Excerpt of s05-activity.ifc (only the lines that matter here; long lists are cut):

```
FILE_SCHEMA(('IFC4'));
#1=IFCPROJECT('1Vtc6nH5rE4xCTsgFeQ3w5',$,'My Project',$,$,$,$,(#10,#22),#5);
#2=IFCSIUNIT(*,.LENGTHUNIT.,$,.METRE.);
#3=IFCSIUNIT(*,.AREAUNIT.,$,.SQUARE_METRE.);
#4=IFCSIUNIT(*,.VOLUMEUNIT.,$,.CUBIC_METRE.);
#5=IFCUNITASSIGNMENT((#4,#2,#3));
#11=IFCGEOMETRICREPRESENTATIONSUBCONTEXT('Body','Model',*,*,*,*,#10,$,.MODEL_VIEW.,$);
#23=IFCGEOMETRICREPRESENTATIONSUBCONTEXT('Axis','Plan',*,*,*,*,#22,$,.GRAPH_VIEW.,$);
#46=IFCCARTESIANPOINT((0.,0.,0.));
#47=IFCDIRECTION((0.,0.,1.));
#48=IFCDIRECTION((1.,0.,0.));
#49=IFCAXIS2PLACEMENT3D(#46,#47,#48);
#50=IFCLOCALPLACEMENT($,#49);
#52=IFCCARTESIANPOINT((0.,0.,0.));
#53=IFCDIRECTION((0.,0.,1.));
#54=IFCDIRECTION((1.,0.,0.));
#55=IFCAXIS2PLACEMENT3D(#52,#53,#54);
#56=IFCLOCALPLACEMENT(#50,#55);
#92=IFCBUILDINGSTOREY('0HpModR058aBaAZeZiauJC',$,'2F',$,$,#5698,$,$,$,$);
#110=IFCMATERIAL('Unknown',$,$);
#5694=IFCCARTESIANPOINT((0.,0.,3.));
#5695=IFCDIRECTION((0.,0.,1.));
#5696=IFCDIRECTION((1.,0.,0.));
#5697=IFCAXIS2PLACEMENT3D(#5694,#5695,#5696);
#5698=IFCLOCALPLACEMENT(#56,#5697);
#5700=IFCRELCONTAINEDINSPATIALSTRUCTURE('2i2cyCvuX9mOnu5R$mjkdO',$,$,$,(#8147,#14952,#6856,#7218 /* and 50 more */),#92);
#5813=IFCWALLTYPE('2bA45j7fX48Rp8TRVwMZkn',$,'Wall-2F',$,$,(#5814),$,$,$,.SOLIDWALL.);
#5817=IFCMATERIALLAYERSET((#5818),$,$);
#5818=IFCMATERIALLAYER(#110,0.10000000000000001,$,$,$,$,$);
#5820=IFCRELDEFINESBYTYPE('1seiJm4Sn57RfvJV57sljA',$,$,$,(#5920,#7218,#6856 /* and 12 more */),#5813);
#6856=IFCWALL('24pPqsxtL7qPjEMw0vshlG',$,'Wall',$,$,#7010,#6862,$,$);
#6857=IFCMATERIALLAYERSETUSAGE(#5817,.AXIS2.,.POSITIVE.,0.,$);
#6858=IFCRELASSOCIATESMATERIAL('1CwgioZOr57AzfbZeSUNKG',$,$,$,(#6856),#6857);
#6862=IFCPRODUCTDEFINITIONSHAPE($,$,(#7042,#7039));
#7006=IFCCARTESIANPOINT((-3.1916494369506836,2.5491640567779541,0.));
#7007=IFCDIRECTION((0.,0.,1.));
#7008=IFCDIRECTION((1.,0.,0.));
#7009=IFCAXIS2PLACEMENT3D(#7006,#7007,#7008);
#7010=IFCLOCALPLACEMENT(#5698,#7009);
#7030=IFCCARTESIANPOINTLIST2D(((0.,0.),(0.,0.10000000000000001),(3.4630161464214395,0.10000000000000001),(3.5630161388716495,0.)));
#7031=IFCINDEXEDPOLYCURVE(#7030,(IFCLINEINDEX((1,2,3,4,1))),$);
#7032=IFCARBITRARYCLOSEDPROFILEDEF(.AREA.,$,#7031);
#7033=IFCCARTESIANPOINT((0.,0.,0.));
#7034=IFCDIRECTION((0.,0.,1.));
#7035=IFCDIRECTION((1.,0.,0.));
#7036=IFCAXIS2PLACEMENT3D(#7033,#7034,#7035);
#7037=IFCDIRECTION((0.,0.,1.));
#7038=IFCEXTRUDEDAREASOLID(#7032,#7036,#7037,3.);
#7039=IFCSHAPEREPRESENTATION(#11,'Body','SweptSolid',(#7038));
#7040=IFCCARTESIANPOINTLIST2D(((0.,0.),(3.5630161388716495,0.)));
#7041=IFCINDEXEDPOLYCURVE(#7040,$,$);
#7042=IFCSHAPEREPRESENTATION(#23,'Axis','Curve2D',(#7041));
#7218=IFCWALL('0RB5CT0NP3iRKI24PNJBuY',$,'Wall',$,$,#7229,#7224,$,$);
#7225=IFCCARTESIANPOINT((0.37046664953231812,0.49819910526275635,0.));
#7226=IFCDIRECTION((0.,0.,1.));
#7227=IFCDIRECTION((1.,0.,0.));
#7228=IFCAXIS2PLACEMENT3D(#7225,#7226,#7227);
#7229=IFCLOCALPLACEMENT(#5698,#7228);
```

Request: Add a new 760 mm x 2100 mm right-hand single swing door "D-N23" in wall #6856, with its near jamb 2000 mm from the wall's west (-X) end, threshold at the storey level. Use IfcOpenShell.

```python
import numpy as np
import ifcopenshell
import ifcopenshell.api.feature
import ifcopenshell.api.geometry
import ifcopenshell.api.root
import ifcopenshell.api.spatial
import ifcopenshell.geom
import ifcopenshell.util.element
import ifcopenshell.util.placement
import ifcopenshell.util.representation
import ifcopenshell.util.shape
import ifcopenshell.util.unit

model = ifcopenshell.open("s05-activity.ifc")
unit_scale = ifcopenshell.util.unit.calculate_unit_scale(model)
settings = ifcopenshell.geom.settings()


def volume(element):
    """Net volume in cubic metres, openings subtracted."""
    shape = ifcopenshell.geom.create_shape(settings, element)
    return ifcopenshell.util.shape.get_volume(shape.geometry)


wall = model.by_id(6856)
storey = ifcopenshell.util.element.get_container(wall, ifc_class="IfcBuildingStorey")
context = ifcopenshell.util.representation.get_context(model, "Model", "Body", "MODEL_VIEW")
before = volume(wall)

width, height, from_end, sill = 0.76, 2.1, 2, 0.0  # metres

# The wall runs along its own X axis, and the end named is its -X end.
wall_shape = ifcopenshell.geom.create_shape(settings, wall)
x, y, z = ifcopenshell.util.shape.get_vertices(wall_shape.geometry).T
start = x.min() + from_end
face, thickness = float(y.min()), float(y.max() - y.min())
wall_matrix = ifcopenshell.util.placement.get_local_placement(wall.ObjectPlacement)
level = ifcopenshell.util.placement.get_local_placement(storey.ObjectPlacement)[2, 3]


def in_wall(x, y):
    """Placement at x, y metres in the wall's axes, at sill height."""
    matrix = wall_matrix.copy()
    matrix[:, 3] = wall_matrix @ np.array([x / unit_scale, y / unit_scale, 0.0, 1.0])
    matrix[2, 3] = level + sill / unit_scale
    return matrix


# Opening: a box that overshoots both wall faces by 50 mm.
opening = ifcopenshell.api.root.create_entity(model, ifc_class="IfcOpeningElement", predefined_type="OPENING")
box = ifcopenshell.api.geometry.add_wall_representation(
    model, context=context, length=width, height=height, thickness=thickness + 0.1
)
ifcopenshell.api.geometry.assign_representation(model, product=opening, representation=box)
ifcopenshell.api.geometry.edit_object_placement(model, product=opening, matrix=in_wall(start, face - 0.05), is_si=False)
ifcopenshell.api.feature.add_feature(model, feature=opening, element=wall)

door = ifcopenshell.api.root.create_entity(model, ifc_class="IfcDoor", name="D-N23", predefined_type="DOOR")
door.OverallWidth, door.OverallHeight = width / unit_scale, height / unit_scale
door.OperationType = "SINGLE_SWING_RIGHT"
body = ifcopenshell.api.geometry.add_door_representation(
    model,
    context=context,
    overall_width=door.OverallWidth,
    overall_height=door.OverallHeight,
    operation_type="SINGLE_SWING_RIGHT",
    lining_properties={"LiningDepth": thickness / unit_scale, "ThresholdDepth": thickness / unit_scale},
)
ifcopenshell.api.geometry.assign_representation(model, product=door, representation=body)
ifcopenshell.api.spatial.assign_container(model, products=[door], relating_structure=storey)
ifcopenshell.api.feature.add_filling(model, opening=opening, element=door)

# The lining spans the wall, so the door starts at the wall face.
ifcopenshell.api.geometry.edit_object_placement(model, product=door, matrix=in_wall(start, face), is_si=False)

after = volume(wall)

print(f"wall volume {before:.3f} -> {after:.3f} m3")

model.write("s05-activity_rev.ifc")
```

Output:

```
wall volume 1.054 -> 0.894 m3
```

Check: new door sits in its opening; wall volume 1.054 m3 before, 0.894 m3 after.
